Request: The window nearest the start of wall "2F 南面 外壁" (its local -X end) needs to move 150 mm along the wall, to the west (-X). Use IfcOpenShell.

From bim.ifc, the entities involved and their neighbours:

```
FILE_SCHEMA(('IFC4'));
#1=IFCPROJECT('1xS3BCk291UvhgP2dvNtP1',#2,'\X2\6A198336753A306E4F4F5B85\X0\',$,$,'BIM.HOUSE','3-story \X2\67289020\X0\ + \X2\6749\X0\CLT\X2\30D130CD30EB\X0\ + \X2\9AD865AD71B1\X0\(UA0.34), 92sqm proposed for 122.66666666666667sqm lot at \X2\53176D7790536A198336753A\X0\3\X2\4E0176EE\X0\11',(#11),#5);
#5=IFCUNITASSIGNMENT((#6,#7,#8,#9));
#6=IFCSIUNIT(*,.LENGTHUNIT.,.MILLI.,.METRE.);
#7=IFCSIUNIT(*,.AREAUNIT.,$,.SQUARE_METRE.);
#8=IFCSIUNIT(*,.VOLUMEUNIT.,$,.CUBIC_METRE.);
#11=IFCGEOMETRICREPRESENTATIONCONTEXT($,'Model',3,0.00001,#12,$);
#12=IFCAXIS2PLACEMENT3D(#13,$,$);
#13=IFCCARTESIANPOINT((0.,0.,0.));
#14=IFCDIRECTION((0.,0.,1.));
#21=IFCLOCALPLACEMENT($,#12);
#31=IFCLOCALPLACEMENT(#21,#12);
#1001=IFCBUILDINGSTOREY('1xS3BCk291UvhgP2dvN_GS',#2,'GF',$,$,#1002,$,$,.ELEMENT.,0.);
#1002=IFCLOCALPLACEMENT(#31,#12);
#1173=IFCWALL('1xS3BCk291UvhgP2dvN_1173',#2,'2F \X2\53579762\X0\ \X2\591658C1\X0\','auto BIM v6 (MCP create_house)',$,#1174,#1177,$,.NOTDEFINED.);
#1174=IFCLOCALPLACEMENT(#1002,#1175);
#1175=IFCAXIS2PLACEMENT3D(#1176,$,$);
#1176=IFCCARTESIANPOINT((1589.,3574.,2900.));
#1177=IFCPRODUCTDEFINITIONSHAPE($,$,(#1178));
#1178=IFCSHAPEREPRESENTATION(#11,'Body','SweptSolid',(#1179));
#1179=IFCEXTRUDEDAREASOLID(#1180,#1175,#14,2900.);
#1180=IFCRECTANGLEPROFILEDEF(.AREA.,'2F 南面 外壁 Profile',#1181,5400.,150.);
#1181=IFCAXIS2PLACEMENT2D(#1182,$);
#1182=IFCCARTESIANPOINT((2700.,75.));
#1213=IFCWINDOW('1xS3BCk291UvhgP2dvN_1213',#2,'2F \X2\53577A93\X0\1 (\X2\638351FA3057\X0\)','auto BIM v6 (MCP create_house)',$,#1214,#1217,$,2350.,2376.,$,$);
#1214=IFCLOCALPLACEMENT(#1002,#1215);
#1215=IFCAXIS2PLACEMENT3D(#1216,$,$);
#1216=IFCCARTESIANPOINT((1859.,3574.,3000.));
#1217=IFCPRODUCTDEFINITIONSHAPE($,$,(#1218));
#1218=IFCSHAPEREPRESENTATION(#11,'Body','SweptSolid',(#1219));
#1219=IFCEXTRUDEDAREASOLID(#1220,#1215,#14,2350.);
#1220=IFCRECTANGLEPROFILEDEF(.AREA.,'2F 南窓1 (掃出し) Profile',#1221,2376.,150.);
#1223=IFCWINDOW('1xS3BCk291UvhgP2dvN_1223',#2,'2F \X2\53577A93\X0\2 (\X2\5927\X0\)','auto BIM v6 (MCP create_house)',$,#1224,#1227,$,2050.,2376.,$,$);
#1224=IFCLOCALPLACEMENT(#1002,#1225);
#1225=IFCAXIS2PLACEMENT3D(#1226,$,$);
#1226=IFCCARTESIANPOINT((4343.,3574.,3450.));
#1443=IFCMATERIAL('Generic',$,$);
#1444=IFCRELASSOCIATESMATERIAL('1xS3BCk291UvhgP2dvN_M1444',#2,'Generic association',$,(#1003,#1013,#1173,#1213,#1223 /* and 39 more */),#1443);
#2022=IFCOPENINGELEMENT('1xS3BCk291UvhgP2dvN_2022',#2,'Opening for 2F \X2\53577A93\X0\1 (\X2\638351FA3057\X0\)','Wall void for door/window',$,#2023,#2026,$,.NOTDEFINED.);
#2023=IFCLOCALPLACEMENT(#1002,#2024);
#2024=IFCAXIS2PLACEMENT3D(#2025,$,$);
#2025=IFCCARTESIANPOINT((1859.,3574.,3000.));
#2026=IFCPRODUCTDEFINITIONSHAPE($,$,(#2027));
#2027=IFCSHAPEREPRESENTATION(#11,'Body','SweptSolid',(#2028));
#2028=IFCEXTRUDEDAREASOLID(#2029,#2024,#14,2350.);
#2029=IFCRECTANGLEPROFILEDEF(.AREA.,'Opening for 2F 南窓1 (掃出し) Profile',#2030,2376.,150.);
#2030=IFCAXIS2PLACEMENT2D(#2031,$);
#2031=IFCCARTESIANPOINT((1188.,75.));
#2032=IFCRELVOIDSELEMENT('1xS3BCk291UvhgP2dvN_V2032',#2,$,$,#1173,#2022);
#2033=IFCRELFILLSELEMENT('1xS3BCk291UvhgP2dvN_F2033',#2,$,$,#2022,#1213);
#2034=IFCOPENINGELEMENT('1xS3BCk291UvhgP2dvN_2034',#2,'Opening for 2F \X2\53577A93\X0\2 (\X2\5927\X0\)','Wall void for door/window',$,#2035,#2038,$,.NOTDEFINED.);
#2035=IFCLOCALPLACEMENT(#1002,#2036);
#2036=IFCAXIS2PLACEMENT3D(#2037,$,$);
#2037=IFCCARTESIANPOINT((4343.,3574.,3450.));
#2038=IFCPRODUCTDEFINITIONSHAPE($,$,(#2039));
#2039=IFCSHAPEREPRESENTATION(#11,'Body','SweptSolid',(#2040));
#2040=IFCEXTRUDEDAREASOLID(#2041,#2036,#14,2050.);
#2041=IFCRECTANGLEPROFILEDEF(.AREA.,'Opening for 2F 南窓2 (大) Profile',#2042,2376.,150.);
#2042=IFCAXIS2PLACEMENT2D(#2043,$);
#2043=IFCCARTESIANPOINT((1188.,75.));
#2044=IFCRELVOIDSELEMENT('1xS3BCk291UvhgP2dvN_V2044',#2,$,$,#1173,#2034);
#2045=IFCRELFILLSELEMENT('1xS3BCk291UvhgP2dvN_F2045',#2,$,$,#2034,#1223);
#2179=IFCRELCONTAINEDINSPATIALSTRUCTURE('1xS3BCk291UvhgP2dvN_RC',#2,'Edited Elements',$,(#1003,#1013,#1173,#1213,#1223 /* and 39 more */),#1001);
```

```python
import ifcopenshell
import ifcopenshell.api.geometry
import ifcopenshell.util.placement

model = ifcopenshell.open("bim.ifc")

window = model.by_guid("1xS3BCk291UvhgP2dvN_1213")
opening = window.FillsVoids[0].RelatingOpeningElement
wall = opening.VoidsElements[0].RelatingBuildingElement

wall_matrix = ifcopenshell.util.placement.get_local_placement(wall.ObjectPlacement)
shift = wall_matrix[:3, 0] * -150.0
before = ifcopenshell.util.placement.get_local_placement(window.ObjectPlacement)[:3, 3].copy()

# The window is not placed relative to its opening, so move both.
for product in (opening, window):
    matrix = ifcopenshell.util.placement.get_local_placement(product.ObjectPlacement)
    matrix[:3, 3] += shift
    ifcopenshell.api.geometry.edit_object_placement(model, product=product, matrix=matrix, is_si=False)

after = ifcopenshell.util.placement.get_local_placement(window.ObjectPlacement)[:3, 3]
print("window moved by", (after - before).round(3) + 0.0)

model.write("bim-out.ifc")
```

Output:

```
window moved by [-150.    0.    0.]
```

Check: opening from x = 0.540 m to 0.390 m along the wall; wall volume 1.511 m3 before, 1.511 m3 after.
